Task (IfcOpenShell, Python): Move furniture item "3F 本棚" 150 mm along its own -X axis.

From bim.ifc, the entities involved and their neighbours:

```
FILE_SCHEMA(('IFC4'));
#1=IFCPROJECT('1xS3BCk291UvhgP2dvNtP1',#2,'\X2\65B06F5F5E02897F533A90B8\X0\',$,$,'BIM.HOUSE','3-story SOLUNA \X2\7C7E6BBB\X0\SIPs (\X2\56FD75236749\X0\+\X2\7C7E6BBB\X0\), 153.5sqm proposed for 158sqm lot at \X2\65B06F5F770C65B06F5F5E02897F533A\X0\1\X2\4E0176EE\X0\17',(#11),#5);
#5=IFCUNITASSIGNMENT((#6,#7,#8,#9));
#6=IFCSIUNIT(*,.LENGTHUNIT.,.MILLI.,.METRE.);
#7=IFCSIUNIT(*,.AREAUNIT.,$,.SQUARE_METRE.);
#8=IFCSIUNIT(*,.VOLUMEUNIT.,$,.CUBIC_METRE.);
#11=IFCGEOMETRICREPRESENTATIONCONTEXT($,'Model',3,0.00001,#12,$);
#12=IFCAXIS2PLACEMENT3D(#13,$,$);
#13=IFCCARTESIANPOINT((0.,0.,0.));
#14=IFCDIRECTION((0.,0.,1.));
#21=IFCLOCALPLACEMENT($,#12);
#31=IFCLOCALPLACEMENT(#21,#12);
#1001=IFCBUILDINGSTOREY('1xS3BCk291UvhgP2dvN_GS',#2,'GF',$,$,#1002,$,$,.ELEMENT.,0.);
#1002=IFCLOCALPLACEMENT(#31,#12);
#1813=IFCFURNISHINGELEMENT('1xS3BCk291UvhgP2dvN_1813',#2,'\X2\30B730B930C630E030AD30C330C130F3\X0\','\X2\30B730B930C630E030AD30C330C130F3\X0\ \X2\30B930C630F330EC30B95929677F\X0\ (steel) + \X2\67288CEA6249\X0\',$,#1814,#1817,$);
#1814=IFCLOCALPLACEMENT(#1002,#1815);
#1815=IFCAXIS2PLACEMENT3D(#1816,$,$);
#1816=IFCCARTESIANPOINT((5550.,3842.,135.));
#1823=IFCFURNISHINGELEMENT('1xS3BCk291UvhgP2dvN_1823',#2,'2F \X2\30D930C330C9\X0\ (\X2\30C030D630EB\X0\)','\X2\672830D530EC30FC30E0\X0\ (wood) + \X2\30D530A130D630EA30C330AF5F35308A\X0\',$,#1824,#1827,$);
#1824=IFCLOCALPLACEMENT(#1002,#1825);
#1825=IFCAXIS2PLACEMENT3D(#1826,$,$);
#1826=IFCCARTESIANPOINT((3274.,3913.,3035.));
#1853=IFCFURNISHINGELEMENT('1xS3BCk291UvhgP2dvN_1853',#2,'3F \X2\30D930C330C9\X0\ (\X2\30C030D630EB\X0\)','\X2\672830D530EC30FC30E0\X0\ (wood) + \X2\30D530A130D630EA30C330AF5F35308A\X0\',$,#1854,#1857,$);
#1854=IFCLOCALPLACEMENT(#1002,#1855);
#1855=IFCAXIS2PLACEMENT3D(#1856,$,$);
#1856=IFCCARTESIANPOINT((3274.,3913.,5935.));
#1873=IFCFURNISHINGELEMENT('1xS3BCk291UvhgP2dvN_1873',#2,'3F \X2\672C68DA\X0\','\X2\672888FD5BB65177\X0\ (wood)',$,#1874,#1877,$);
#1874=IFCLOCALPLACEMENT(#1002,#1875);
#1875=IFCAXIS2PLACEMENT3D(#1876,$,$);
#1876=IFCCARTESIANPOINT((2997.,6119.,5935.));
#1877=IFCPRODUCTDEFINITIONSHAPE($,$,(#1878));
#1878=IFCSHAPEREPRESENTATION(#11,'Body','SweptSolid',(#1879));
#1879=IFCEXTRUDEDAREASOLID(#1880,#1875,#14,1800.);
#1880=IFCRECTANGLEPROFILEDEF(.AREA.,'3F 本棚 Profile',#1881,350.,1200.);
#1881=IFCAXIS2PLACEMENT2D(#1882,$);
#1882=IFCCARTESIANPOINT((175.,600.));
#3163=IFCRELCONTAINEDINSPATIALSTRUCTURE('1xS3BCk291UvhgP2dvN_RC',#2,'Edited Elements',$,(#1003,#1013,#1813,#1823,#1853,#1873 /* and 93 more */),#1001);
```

```python
import ifcopenshell
import ifcopenshell.api.geometry
import ifcopenshell.util.placement
import ifcopenshell.util.unit

model = ifcopenshell.open("bim.ifc")
unit_scale = ifcopenshell.util.unit.calculate_unit_scale(model)

item = model.by_guid("1xS3BCk291UvhgP2dvN_1873")
matrix = ifcopenshell.util.placement.get_local_placement(item.ObjectPlacement)
matrix[:3, 3] -= matrix[:3, 0] * 0.15 / unit_scale
ifcopenshell.api.geometry.edit_object_placement(model, product=item, matrix=matrix, is_si=False)

print(ifcopenshell.util.placement.get_local_placement(item.ObjectPlacement).round(3) + 0.0)

model.write("bim-out.ifc")
```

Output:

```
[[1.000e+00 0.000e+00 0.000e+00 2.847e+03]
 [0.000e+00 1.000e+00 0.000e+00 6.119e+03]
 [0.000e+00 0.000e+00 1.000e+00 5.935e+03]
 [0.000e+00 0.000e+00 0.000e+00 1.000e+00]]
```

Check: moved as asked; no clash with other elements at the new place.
